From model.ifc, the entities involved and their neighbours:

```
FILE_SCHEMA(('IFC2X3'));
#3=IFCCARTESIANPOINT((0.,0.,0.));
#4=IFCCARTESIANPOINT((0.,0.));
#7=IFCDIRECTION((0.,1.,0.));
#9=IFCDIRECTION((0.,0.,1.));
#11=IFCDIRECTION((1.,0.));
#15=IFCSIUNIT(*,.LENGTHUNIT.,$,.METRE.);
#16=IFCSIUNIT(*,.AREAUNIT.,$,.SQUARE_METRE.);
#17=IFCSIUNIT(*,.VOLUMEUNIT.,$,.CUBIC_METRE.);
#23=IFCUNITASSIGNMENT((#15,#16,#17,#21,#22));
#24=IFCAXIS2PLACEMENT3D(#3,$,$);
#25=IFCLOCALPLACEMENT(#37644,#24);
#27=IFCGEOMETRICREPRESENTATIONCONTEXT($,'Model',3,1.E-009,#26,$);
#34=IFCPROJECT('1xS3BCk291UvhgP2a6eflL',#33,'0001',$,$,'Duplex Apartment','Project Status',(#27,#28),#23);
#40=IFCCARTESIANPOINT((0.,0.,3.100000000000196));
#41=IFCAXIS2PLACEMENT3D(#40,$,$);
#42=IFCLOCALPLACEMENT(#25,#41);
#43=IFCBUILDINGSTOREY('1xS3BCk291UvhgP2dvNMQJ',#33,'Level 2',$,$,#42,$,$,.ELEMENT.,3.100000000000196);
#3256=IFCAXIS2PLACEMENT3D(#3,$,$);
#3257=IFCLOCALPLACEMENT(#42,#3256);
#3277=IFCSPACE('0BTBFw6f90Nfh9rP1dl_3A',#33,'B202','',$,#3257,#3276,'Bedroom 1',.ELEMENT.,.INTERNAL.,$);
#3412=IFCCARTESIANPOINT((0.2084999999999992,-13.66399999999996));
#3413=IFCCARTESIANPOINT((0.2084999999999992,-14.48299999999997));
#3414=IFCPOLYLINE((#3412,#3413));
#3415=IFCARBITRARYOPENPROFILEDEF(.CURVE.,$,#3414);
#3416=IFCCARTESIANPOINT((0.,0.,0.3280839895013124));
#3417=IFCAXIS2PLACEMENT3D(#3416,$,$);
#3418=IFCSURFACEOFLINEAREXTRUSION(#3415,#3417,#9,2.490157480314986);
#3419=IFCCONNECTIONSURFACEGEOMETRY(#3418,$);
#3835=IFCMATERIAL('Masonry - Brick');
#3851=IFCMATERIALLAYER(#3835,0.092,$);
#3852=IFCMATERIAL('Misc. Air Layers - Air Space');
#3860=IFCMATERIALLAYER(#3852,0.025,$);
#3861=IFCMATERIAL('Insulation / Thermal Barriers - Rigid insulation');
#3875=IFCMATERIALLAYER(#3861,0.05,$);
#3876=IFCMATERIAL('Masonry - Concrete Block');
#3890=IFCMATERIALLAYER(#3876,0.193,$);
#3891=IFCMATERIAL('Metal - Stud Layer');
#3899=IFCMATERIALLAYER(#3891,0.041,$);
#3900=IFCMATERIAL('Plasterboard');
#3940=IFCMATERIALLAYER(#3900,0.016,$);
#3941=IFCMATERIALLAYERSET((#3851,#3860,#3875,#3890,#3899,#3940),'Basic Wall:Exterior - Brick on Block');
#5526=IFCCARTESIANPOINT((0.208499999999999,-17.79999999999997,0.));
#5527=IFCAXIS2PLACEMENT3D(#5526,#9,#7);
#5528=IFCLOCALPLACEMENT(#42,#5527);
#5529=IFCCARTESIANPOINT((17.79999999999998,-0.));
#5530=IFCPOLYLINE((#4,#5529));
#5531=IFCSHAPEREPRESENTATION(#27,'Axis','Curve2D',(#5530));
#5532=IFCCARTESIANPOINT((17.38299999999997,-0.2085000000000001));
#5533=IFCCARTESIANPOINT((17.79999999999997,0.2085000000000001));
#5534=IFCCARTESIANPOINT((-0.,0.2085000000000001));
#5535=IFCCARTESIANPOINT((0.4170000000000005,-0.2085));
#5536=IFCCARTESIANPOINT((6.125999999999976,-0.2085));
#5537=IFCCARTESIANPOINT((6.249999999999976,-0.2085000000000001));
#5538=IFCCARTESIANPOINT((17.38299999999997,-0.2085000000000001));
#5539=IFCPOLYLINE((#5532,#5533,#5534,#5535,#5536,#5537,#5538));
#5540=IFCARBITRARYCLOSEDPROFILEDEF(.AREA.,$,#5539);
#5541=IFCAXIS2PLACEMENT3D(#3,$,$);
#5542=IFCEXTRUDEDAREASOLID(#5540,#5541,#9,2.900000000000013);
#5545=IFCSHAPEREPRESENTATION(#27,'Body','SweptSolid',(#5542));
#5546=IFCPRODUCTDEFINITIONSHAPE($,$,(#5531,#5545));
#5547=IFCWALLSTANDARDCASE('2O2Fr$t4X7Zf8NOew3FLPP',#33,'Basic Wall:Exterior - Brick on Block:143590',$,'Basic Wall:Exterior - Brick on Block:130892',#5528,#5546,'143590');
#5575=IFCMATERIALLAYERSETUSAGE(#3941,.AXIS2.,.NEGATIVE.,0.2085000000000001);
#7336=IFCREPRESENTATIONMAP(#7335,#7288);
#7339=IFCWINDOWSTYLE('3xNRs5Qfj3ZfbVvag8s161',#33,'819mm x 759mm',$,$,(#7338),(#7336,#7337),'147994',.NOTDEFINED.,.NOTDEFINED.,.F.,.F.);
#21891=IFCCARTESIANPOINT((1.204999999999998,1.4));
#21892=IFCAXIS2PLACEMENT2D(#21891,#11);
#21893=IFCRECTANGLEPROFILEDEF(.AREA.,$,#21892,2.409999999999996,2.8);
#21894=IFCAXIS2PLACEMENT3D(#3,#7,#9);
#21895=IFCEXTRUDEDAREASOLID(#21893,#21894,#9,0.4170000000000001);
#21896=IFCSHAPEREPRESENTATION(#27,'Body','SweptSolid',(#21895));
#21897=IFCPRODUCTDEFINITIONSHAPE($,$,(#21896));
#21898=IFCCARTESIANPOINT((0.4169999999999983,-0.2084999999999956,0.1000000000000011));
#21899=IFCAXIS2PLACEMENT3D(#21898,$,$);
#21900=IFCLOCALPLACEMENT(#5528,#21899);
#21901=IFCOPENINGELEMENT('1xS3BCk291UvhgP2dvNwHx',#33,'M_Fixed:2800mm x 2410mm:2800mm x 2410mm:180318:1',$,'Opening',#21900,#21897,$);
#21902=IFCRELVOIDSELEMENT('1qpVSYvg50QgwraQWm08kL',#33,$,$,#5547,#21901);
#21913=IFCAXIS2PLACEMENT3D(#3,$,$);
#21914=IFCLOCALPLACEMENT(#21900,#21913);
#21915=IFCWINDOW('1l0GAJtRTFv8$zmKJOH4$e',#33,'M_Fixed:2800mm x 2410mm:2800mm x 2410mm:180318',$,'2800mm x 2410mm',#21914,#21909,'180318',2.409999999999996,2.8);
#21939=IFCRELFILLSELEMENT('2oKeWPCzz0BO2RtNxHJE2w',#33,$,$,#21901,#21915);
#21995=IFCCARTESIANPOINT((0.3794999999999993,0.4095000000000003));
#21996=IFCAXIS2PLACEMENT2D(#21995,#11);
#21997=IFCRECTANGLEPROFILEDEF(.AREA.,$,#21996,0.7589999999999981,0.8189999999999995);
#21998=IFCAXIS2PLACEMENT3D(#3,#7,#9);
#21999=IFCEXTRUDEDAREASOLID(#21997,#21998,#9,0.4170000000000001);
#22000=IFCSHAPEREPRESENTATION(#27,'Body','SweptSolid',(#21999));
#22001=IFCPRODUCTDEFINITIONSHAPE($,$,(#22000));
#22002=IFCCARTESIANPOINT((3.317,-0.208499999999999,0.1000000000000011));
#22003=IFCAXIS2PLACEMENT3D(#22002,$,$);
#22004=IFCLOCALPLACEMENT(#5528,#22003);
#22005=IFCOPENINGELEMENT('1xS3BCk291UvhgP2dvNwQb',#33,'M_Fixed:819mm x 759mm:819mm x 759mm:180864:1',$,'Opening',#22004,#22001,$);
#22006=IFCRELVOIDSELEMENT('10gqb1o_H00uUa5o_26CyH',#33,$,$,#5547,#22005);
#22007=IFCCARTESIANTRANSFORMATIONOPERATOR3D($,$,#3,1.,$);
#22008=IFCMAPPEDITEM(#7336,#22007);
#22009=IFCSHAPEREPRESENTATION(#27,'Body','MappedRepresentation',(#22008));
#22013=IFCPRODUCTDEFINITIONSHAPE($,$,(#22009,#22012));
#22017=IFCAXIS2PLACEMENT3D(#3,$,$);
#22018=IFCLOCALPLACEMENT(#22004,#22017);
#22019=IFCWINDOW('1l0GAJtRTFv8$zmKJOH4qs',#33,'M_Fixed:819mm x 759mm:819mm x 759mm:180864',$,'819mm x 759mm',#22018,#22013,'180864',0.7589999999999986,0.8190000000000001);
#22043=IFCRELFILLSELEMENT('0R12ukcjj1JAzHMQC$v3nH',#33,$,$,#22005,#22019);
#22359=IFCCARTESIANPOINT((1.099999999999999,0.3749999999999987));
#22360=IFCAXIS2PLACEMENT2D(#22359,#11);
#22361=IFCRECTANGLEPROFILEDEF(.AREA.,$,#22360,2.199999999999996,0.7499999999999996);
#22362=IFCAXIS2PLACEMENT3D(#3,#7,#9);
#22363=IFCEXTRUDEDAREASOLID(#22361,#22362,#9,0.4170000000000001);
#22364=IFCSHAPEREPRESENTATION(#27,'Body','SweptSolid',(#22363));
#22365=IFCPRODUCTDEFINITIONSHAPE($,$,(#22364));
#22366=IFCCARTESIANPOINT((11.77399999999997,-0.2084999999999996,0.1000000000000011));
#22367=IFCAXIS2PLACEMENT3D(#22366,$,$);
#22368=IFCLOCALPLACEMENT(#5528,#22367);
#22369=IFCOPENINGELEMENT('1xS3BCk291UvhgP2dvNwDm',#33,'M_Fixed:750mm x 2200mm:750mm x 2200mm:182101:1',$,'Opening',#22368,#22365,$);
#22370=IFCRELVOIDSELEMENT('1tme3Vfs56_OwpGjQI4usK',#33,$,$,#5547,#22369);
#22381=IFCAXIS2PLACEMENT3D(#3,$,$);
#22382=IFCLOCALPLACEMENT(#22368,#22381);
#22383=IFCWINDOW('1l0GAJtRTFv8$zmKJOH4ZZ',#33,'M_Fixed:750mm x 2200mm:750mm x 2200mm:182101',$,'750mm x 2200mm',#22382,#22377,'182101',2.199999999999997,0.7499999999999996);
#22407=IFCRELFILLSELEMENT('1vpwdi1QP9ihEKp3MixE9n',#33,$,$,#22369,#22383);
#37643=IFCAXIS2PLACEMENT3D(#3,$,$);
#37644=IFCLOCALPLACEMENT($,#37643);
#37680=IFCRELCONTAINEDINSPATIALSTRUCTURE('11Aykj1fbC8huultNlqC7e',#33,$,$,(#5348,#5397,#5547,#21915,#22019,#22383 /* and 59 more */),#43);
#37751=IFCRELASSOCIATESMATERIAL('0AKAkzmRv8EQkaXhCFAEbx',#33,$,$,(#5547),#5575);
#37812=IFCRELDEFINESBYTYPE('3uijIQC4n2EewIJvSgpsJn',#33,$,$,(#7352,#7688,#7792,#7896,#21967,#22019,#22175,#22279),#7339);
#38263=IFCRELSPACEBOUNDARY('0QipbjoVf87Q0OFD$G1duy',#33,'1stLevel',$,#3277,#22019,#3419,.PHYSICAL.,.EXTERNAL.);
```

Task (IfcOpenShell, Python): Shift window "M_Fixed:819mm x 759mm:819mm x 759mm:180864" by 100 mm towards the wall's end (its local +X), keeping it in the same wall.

```python
import numpy as np
import ifcopenshell
import ifcopenshell.api.geometry
import ifcopenshell.util.placement
import ifcopenshell.util.unit

model = ifcopenshell.open("model.ifc")
unit_scale = ifcopenshell.util.unit.calculate_unit_scale(model)

window = model.by_guid("1l0GAJtRTFv8$zmKJOH4qs")
opening = window.FillsVoids[0].RelatingOpeningElement
wall = opening.VoidsElements[0].RelatingBuildingElement

wall_matrix = ifcopenshell.util.placement.get_local_placement(wall.ObjectPlacement)
shift = wall_matrix[:3, 0] * 0.1 / unit_scale
before = ifcopenshell.util.placement.get_local_placement(window.ObjectPlacement)[:3, 3].copy()

# The window is placed relative to its opening, so it follows when the opening moves.
matrix = ifcopenshell.util.placement.get_local_placement(opening.ObjectPlacement)
matrix[:3, 3] += shift
ifcopenshell.api.geometry.edit_object_placement(
    model, product=opening, matrix=matrix, is_si=False, should_transform_children=True
)

# Space boundary surfaces are stored in each space's coordinates; move them too.
for rel in window.ProvidesBoundaries:
    if not rel.ConnectionGeometry:
        continue
    surface = rel.ConnectionGeometry.SurfaceOnRelatingElement
    space_matrix = ifcopenshell.util.placement.get_local_placement(rel.RelatingSpace.ObjectPlacement)
    point = np.array(surface.Position.Location.Coordinates) + space_matrix[:3, :3].T @ shift
    surface.Position = model.createIfcAxis2Placement3D(
        model.createIfcCartesianPoint(point.tolist()), surface.Position.Axis, surface.Position.RefDirection
    )

after = ifcopenshell.util.placement.get_local_placement(window.ObjectPlacement)[:3, 3]
print("window moved by", (after - before).round(3) + 0.0)

model.write("model-out.ifc")
```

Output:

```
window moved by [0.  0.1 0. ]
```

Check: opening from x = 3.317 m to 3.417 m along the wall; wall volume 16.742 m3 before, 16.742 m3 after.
